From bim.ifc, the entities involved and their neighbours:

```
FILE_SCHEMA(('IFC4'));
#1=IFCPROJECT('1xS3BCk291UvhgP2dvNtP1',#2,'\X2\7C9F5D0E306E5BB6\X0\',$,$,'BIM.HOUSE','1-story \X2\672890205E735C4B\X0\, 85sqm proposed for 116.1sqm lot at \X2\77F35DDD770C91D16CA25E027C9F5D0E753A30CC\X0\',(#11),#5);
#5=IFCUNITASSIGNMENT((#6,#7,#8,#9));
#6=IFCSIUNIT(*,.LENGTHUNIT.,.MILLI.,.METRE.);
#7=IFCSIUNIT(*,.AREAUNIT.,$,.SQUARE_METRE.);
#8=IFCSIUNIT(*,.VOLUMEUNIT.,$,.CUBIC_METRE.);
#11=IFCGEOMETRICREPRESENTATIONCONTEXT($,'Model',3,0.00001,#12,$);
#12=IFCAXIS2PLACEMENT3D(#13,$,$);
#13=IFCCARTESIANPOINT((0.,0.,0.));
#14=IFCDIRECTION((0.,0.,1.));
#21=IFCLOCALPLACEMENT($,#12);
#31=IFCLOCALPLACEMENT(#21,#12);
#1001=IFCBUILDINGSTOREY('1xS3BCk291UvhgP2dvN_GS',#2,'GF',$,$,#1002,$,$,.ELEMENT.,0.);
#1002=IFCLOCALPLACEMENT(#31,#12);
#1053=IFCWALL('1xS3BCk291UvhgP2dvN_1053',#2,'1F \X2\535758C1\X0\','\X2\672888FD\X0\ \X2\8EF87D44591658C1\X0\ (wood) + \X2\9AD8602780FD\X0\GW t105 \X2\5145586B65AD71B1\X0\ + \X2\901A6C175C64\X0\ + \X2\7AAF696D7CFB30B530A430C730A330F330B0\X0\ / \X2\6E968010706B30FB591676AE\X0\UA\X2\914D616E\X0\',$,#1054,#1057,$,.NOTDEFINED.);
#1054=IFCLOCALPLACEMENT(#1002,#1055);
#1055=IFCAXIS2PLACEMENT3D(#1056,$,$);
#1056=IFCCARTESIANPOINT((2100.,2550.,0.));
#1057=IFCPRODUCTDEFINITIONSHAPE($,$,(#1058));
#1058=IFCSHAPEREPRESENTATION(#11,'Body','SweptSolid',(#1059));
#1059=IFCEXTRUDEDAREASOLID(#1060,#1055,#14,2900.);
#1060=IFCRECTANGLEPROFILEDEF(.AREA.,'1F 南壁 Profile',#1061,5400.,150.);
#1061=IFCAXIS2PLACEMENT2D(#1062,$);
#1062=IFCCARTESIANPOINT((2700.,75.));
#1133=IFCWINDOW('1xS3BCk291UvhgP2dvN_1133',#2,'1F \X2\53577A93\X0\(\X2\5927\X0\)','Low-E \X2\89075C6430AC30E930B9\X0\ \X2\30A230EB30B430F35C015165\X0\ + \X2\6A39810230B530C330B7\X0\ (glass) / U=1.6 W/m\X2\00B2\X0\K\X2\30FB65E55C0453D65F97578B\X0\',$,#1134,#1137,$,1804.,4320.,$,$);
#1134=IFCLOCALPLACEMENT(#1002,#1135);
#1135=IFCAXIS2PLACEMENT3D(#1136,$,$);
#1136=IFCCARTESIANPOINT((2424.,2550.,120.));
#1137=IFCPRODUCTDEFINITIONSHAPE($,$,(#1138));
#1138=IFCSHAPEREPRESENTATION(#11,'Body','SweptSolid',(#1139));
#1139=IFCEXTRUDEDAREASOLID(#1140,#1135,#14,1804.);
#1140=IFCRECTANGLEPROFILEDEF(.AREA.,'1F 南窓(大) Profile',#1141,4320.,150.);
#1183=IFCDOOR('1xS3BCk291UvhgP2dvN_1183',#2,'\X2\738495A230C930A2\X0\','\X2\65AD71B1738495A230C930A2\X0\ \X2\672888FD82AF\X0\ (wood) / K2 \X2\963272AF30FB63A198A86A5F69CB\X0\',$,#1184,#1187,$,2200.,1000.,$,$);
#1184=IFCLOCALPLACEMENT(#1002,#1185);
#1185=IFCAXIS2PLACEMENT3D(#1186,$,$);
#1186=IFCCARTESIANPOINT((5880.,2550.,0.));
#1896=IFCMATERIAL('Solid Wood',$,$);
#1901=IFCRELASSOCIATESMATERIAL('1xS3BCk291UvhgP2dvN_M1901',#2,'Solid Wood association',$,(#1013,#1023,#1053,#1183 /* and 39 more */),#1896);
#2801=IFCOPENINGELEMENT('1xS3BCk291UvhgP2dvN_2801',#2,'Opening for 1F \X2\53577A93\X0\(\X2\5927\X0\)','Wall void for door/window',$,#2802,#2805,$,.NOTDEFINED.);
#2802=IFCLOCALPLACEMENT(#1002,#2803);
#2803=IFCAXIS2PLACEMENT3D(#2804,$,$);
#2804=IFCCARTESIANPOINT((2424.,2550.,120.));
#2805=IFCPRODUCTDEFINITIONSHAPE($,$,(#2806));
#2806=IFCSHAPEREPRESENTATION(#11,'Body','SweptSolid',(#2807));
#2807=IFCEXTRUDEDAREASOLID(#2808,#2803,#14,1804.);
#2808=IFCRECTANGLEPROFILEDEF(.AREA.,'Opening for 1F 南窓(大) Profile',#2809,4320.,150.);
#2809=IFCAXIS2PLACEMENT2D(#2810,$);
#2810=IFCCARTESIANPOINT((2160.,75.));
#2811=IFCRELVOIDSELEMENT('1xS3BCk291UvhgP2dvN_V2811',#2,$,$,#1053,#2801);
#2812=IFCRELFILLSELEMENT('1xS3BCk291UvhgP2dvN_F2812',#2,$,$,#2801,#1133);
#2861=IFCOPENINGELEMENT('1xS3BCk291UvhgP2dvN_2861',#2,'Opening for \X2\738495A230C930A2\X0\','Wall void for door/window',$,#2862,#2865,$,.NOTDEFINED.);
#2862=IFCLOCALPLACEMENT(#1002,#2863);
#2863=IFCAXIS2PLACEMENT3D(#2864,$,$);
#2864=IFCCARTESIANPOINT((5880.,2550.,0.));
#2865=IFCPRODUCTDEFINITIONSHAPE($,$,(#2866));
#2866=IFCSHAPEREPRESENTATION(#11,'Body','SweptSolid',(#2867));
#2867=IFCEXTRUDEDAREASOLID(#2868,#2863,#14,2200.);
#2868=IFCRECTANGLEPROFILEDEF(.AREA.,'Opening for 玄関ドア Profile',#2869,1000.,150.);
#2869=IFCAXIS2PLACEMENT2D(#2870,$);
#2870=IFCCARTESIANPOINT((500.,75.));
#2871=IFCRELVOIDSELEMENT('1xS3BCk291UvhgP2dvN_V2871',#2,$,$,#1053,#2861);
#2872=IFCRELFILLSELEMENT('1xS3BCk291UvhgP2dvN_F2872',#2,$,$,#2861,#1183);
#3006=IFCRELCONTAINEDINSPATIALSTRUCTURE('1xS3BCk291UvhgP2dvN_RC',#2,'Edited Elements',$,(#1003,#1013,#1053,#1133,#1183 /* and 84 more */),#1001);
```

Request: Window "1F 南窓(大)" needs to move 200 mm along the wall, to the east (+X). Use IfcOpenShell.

```python
import ifcopenshell
import ifcopenshell.api.geometry
import ifcopenshell.util.placement

model = ifcopenshell.open("bim.ifc")

window = model.by_id(1133)
opening = window.FillsVoids[0].RelatingOpeningElement
wall = opening.VoidsElements[0].RelatingBuildingElement

wall_matrix = ifcopenshell.util.placement.get_local_placement(wall.ObjectPlacement)
shift = wall_matrix[:3, 0] * 200.0
before = ifcopenshell.util.placement.get_local_placement(window.ObjectPlacement)[:3, 3].copy()

# The window is not placed relative to its opening, so move both.
for product in (opening, window):
    matrix = ifcopenshell.util.placement.get_local_placement(product.ObjectPlacement)
    matrix[:3, 3] += shift
    ifcopenshell.api.geometry.edit_object_placement(model, product=product, matrix=matrix, is_si=False)

after = ifcopenshell.util.placement.get_local_placement(window.ObjectPlacement)[:3, 3]
print("window moved by", (after - before).round(3) + 0.0)

model.write("bim_v2.ifc")
```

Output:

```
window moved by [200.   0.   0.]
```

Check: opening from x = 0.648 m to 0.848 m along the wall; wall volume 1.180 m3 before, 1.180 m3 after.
